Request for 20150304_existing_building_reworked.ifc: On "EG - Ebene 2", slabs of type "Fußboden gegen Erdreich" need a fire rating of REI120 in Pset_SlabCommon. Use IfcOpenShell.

First a look at what the model holds.

```python
import ifcopenshell
import ifcopenshell.util.element

model = ifcopenshell.open("20150304_existing_building_reworked.ifc")
print(model.schema)
storey = next(s for s in model.by_type("IfcBuildingStorey") if s.Name == "EG - Ebene 2")
slabs = [e for e in ifcopenshell.util.element.get_decomposition(storey) if e.is_a("IfcSlab")]
seen = {}
for e in slabs:
    element_type = ifcopenshell.util.element.get_type(e)
    key = (element_type.Name if element_type != e and element_type else None, ifcopenshell.util.element.get_pset(e, "Pset_SlabCommon", "FireRating"))
    seen[key] = seen.get(key, 0) + 1
for (name, value), count in sorted(seen.items(), key=str):
    print(count, "x", name, "|", value)
```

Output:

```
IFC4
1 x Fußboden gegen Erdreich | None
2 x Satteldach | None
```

```python
import ifcopenshell
import ifcopenshell.api.pset
import ifcopenshell.util.element

model = ifcopenshell.open("20150304_existing_building_reworked.ifc")

storey = next(s for s in model.by_type("IfcBuildingStorey") if s.Name == "EG - Ebene 2")
slabs = [e for e in ifcopenshell.util.element.get_decomposition(storey) if e.is_a("IfcSlab")]

count = 0
for e in slabs:
    element_type = ifcopenshell.util.element.get_type(e)
    if element_type in (None, e) or element_type.Name != "Fußboden gegen Erdreich":
        continue
    # add_pset returns the element's existing set when there is one.
    pset = ifcopenshell.api.pset.add_pset(model, product=e, name="Pset_SlabCommon")
    ifcopenshell.api.pset.edit_pset(model, pset=pset, properties={"FireRating": "REI120"})
    count += 1

print(count, "slabs updated")

model.write("20150304_existing_building_reworked_edited.ifc")
```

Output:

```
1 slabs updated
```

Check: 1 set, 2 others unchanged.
